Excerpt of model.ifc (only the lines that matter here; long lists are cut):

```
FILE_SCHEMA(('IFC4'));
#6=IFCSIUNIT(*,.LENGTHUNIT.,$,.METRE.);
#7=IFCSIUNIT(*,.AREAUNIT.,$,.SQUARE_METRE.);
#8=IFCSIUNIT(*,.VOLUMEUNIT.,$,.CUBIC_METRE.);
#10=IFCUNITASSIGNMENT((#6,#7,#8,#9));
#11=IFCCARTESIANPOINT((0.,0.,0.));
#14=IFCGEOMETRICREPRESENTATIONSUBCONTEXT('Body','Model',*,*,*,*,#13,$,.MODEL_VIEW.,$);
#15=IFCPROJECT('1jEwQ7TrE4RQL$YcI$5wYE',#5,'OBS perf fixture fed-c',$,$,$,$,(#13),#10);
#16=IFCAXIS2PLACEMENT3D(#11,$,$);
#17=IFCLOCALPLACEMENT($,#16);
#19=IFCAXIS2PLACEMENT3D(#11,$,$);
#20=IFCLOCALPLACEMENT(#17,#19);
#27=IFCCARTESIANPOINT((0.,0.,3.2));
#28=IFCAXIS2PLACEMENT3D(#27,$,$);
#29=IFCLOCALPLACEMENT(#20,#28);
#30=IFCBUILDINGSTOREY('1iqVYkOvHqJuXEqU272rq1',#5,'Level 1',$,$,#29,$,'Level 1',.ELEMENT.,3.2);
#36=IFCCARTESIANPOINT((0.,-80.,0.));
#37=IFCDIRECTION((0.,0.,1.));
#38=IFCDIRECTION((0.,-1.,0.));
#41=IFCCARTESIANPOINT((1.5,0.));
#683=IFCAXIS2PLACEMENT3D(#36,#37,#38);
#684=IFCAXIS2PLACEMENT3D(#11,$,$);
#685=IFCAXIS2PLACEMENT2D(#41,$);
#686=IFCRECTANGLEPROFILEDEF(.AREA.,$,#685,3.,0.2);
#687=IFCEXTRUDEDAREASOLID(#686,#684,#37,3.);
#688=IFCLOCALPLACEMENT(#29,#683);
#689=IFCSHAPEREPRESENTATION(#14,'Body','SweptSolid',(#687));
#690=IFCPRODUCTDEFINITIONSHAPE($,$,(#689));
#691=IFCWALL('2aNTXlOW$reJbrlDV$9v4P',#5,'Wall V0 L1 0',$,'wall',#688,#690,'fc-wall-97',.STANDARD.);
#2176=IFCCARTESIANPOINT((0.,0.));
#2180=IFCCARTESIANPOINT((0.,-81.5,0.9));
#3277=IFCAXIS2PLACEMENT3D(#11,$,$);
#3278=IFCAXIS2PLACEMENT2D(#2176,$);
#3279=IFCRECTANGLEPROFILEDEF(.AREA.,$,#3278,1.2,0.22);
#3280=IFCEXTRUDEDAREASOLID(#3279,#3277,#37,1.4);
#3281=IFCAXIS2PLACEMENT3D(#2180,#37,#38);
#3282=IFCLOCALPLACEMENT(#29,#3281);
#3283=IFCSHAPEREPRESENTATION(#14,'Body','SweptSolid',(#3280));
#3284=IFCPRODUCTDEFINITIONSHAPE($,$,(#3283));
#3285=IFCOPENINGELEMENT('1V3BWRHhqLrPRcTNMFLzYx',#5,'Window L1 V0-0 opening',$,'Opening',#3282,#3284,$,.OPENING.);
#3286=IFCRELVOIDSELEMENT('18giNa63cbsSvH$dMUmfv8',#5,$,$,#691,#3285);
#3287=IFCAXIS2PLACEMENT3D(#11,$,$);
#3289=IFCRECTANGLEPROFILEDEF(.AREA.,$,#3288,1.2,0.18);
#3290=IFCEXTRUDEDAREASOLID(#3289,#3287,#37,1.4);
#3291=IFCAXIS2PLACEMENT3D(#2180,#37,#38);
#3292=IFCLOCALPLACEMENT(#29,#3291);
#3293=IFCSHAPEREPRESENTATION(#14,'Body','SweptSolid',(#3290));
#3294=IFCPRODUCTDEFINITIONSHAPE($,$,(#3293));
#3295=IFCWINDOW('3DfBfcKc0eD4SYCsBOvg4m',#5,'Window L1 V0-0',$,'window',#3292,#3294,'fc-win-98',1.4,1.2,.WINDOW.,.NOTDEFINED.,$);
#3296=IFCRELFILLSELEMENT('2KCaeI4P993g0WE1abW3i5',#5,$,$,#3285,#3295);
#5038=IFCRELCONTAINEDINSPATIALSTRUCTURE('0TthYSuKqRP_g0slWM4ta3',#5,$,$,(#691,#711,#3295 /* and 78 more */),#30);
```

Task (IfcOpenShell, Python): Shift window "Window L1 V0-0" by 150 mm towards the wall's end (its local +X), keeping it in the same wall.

```python
import ifcopenshell
import ifcopenshell.api.geometry
import ifcopenshell.util.placement
import ifcopenshell.util.unit

model = ifcopenshell.open("model.ifc")
unit_scale = ifcopenshell.util.unit.calculate_unit_scale(model)

window = model.by_guid("3DfBfcKc0eD4SYCsBOvg4m")
opening = window.FillsVoids[0].RelatingOpeningElement
wall = opening.VoidsElements[0].RelatingBuildingElement

wall_matrix = ifcopenshell.util.placement.get_local_placement(wall.ObjectPlacement)
shift = wall_matrix[:3, 0] * 0.15 / unit_scale
before = ifcopenshell.util.placement.get_local_placement(window.ObjectPlacement)[:3, 3].copy()

# The window is not placed relative to its opening, so move both.
for product in (opening, window):
    matrix = ifcopenshell.util.placement.get_local_placement(product.ObjectPlacement)
    matrix[:3, 3] += shift
    ifcopenshell.api.geometry.edit_object_placement(model, product=product, matrix=matrix, is_si=False)

after = ifcopenshell.util.placement.get_local_placement(window.ObjectPlacement)[:3, 3]
print("window moved by", (after - before).round(3) + 0.0)

model.write("model-out.ifc")
```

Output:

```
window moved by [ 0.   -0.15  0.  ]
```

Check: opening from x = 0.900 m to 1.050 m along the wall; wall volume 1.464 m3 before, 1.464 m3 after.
